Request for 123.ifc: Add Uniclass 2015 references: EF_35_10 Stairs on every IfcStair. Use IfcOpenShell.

First a look at what the model holds.

```python
import ifcopenshell

model = ifcopenshell.open("123.ifc")
print(model.schema)
print("classifications:", [c.Name for c in model.by_type("IfcClassification")])
for ifc_class in ("IfcDoor", "IfcRoof", "IfcStair", "IfcWall", "IfcWindow"):
    print(ifc_class, len(model.by_type(ifc_class)))
```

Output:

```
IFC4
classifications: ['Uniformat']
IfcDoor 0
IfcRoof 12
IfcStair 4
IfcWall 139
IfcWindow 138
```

```python
import ifcopenshell
import ifcopenshell.api.classification

model = ifcopenshell.open("123.ifc")

system = ifcopenshell.api.classification.add_classification(model, classification="Uniclass 2015")

codes = {
    "IfcStair": ("EF_35_10", "Stairs"),
}
for ifc_class, (code, name) in codes.items():
    products = model.by_type(ifc_class)
    ifcopenshell.api.classification.add_reference(
        model, products=products, classification=system, identification=code, name=name
    )
    print(code, len(products))

model.write("123_edited.ifc")
```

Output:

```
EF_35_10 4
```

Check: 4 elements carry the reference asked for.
